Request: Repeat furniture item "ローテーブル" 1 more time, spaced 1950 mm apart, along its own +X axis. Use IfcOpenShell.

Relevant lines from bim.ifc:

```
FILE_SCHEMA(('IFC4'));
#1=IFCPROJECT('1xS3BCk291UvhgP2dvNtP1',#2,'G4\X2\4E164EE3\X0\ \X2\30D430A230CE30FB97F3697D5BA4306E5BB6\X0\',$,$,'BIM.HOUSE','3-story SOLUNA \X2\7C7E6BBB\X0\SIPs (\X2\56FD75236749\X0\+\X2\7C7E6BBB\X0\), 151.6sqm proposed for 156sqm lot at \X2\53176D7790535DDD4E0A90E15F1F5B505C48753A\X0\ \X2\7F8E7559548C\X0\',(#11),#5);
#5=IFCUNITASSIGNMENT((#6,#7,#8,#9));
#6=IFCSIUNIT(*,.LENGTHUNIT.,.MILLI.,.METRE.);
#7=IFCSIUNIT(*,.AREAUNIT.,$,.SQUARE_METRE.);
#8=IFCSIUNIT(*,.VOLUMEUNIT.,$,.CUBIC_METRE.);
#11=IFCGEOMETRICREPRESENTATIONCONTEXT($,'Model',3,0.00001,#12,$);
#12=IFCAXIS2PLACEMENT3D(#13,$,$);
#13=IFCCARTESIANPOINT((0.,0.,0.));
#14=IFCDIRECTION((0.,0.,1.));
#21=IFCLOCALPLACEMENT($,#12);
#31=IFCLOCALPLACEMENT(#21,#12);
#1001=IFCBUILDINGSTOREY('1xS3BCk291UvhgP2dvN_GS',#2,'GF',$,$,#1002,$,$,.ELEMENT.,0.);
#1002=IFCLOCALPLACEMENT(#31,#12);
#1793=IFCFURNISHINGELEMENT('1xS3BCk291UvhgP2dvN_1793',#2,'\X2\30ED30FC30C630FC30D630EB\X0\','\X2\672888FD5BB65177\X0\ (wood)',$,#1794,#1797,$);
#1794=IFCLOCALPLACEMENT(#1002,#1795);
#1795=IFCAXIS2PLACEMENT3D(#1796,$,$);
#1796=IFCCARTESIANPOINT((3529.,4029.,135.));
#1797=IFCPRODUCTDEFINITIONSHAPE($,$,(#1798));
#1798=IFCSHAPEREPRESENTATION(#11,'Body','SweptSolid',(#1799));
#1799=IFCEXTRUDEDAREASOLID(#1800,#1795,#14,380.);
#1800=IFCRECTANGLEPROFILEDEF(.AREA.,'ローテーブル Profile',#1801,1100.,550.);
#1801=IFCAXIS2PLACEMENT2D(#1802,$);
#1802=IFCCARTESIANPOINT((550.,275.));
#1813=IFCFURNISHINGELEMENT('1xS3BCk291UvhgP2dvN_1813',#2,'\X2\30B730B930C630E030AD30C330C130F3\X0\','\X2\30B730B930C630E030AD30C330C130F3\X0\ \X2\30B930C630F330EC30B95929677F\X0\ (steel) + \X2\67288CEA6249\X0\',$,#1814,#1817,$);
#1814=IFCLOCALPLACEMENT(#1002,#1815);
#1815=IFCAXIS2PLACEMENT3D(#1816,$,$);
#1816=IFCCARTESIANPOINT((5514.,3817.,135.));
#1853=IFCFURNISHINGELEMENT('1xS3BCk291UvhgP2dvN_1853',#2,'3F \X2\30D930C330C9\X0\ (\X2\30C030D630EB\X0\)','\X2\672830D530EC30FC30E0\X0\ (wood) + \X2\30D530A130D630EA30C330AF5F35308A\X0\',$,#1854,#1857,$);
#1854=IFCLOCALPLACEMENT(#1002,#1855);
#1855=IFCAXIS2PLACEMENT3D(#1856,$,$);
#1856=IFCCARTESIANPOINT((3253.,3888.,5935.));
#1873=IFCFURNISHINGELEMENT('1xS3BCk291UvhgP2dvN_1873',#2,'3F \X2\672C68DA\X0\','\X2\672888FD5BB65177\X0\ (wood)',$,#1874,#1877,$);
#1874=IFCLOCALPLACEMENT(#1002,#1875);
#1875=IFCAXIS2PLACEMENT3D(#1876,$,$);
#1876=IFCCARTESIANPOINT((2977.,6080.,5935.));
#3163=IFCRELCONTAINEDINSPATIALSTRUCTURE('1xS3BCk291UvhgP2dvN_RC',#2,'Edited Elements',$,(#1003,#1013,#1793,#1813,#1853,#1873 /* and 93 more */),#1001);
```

```python
import ifcopenshell
import ifcopenshell.api.geometry
import ifcopenshell.api.root
import ifcopenshell.util.element
import ifcopenshell.util.placement
import ifcopenshell.util.unit

model = ifcopenshell.open("bim.ifc")
unit_scale = ifcopenshell.util.unit.calculate_unit_scale(model)


def reuse_history(source, copy):
    """copy_class also copies each property set's owner history, people and application; keep the originals."""
    for rel in copy.IsDefinedBy:
        if rel.is_a("IfcRelDefinesByProperties") and (history := rel.RelatingPropertyDefinition.OwnerHistory):
            rel.RelatingPropertyDefinition.OwnerHistory = source.OwnerHistory
            ifcopenshell.util.element.remove_deep2(model, history)


source = model.by_id(1793)
base = ifcopenshell.util.placement.get_local_placement(source.ObjectPlacement)
step = base[:3, 0] * 1.95 / unit_scale

for i in range(1, 2):
    copy = ifcopenshell.api.root.copy_class(model, product=source)
    copy.Representation = ifcopenshell.util.element.copy_deep(
        model, source.Representation, exclude=["IfcGeometricRepresentationContext", "IfcRepresentationMap"]
    )
    reuse_history(source, copy)
    matrix = base.copy()
    matrix[:3, 3] += i * step
    print("added at", matrix[:3, 3].round(3) + 0.0)
    ifcopenshell.api.geometry.edit_object_placement(model, product=copy, matrix=matrix, is_si=False)

model.write("bim_edited.ifc")
```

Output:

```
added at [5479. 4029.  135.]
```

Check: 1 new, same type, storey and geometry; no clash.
